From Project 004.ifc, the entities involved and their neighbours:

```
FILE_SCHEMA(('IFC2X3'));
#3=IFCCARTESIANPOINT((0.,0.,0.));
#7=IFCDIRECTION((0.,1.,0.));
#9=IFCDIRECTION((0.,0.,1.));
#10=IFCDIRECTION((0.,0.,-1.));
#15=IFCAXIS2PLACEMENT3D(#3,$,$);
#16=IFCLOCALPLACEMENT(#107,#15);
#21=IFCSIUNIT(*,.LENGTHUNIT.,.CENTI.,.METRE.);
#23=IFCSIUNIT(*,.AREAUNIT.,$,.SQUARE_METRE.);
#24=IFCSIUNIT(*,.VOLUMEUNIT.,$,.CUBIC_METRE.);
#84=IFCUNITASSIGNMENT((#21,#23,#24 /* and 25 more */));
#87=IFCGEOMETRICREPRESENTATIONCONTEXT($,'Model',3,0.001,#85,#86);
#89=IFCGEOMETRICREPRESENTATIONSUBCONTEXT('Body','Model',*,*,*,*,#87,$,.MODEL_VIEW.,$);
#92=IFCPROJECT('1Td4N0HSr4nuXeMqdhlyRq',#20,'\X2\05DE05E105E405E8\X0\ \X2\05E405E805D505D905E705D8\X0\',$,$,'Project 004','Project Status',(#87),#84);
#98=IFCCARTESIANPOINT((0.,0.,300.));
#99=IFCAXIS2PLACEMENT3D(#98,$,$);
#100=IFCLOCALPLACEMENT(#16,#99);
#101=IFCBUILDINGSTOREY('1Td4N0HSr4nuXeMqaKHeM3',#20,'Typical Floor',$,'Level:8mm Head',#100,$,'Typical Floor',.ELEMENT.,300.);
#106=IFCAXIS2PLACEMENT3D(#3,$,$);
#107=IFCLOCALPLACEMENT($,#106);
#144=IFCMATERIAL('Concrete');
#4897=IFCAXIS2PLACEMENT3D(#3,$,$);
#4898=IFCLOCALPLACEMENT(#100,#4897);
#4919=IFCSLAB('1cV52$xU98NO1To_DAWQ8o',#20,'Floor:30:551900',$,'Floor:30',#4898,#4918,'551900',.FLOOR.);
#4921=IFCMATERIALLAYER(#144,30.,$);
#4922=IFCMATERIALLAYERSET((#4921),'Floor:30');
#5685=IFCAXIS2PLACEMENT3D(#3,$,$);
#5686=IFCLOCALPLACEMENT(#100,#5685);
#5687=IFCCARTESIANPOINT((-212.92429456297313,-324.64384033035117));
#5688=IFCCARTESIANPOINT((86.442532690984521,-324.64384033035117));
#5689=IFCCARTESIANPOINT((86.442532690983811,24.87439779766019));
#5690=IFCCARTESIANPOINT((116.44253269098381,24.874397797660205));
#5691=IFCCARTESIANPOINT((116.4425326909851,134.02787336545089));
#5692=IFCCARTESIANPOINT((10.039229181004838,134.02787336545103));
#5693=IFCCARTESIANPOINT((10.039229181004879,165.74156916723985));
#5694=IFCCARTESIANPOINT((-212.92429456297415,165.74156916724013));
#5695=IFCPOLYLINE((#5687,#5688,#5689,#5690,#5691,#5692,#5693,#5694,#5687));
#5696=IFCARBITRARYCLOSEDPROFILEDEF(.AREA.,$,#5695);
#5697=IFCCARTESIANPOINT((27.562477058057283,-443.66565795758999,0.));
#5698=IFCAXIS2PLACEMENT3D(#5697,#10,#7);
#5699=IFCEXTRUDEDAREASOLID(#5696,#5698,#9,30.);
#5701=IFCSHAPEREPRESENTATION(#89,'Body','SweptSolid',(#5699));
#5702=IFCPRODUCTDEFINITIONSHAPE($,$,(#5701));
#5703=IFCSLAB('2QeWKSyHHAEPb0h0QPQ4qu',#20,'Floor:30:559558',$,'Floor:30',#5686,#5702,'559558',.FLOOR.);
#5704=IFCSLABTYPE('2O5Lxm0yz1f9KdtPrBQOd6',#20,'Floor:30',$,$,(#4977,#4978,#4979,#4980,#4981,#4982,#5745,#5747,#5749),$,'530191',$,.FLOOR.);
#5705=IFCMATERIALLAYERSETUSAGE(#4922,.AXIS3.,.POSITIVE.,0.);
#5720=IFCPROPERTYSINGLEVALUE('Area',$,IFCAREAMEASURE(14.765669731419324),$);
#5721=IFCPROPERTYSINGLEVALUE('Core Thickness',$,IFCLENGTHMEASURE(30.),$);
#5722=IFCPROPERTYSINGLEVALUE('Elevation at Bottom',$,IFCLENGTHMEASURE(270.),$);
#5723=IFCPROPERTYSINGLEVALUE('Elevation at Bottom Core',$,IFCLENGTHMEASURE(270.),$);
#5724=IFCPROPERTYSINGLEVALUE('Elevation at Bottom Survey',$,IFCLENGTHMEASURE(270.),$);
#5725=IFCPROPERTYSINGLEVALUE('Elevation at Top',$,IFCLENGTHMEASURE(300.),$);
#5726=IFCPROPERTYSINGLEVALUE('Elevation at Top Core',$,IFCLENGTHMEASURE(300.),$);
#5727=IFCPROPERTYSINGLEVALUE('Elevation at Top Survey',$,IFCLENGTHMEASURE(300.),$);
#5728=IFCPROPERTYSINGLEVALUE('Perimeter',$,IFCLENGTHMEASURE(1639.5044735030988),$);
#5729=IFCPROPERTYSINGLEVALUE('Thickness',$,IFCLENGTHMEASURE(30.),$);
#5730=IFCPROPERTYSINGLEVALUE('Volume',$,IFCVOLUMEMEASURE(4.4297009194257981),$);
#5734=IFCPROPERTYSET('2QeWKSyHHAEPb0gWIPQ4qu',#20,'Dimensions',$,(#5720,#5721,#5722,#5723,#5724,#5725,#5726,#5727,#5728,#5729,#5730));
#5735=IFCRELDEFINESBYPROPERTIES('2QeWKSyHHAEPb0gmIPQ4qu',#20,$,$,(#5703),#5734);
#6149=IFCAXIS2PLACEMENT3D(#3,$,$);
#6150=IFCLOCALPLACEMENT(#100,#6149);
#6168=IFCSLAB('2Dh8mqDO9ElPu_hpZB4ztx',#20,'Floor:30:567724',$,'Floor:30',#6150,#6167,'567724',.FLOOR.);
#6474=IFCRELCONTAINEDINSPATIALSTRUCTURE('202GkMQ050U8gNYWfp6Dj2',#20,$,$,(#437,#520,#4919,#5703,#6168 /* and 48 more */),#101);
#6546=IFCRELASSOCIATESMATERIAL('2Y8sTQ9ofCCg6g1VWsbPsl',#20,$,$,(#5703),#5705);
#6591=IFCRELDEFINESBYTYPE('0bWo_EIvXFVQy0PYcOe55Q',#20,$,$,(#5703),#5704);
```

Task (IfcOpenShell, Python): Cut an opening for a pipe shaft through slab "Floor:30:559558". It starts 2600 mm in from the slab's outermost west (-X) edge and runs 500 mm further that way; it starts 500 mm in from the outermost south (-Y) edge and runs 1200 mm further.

```python
import numpy as np
import ifcopenshell
import ifcopenshell.api.feature
import ifcopenshell.api.geometry
import ifcopenshell.api.pset
import ifcopenshell.api.root
import ifcopenshell.geom
import ifcopenshell.util.element
import ifcopenshell.util.placement
import ifcopenshell.util.representation
import ifcopenshell.util.shape
import ifcopenshell.util.unit

model = ifcopenshell.open("Project 004.ifc")
unit_scale = ifcopenshell.util.unit.calculate_unit_scale(model)
area_scale = ifcopenshell.util.unit.calculate_unit_scale(model, "AREAUNIT")
volume_scale = ifcopenshell.util.unit.calculate_unit_scale(model, "VOLUMEUNIT")
settings = ifcopenshell.geom.settings()


def volume(element):
    """Net volume in cubic metres, openings subtracted."""
    shape = ifcopenshell.geom.create_shape(settings, element)
    return ifcopenshell.util.shape.get_volume(shape.geometry)


slab = model.by_guid("2QeWKSyHHAEPb0h0QPQ4qu")
before = volume(slab)

# Extent in the slab's own axes, in metres. The edges named are its -X and -Y sides.
slab_shape = ifcopenshell.geom.create_shape(settings, slab)
vertices = ifcopenshell.util.shape.get_vertices(slab_shape.geometry)
x_min, y_min, bottom = vertices.min(axis=0)
top = vertices[:, 2].max()

opening = ifcopenshell.api.root.create_entity(model, ifc_class="IfcOpeningElement", name="Pipe shaft opening")
context = ifcopenshell.util.representation.get_context(model, "Model", "Body", "MODEL_VIEW")
width, depth = 0.5, 1.2
outline = [(0.0, 0.0), (width, 0.0), (width, depth), (0.0, depth), (0.0, 0.0)]
# Overshoot both faces by 50 mm so the cut is clean.
shape = ifcopenshell.api.geometry.add_slab_representation(
    model, context=context, depth=top - bottom + 0.1, polyline=outline
)
ifcopenshell.api.geometry.assign_representation(model, product=opening, representation=shape)

matrix = ifcopenshell.util.placement.get_local_placement(slab.ObjectPlacement)
matrix[:, 3] = matrix @ np.append(np.array([x_min + 2.6, y_min + 0.5, bottom - 0.05]) / unit_scale, 1.0)
ifcopenshell.api.geometry.edit_object_placement(model, product=opening, matrix=matrix, is_si=False)
ifcopenshell.api.feature.add_feature(model, feature=opening, element=slab)

after = volume(slab)

# Update the slab's stored quantities.
pset = model.by_id(ifcopenshell.util.element.get_pset(slab, "Dimensions", should_inherit=False)["id"])
ifcopenshell.api.pset.edit_pset(model, pset=pset, properties={
    "Area": model.create_entity("IfcAreaMeasure", after / (top - bottom) / area_scale),
    "Volume": model.create_entity("IfcVolumeMeasure", after / volume_scale),
})

print(f"slab volume {before:.3f} -> {after:.3f} m3")

model.write("Project 004_v2.ifc")
```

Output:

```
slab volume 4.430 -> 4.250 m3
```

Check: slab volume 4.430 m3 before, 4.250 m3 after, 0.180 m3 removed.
